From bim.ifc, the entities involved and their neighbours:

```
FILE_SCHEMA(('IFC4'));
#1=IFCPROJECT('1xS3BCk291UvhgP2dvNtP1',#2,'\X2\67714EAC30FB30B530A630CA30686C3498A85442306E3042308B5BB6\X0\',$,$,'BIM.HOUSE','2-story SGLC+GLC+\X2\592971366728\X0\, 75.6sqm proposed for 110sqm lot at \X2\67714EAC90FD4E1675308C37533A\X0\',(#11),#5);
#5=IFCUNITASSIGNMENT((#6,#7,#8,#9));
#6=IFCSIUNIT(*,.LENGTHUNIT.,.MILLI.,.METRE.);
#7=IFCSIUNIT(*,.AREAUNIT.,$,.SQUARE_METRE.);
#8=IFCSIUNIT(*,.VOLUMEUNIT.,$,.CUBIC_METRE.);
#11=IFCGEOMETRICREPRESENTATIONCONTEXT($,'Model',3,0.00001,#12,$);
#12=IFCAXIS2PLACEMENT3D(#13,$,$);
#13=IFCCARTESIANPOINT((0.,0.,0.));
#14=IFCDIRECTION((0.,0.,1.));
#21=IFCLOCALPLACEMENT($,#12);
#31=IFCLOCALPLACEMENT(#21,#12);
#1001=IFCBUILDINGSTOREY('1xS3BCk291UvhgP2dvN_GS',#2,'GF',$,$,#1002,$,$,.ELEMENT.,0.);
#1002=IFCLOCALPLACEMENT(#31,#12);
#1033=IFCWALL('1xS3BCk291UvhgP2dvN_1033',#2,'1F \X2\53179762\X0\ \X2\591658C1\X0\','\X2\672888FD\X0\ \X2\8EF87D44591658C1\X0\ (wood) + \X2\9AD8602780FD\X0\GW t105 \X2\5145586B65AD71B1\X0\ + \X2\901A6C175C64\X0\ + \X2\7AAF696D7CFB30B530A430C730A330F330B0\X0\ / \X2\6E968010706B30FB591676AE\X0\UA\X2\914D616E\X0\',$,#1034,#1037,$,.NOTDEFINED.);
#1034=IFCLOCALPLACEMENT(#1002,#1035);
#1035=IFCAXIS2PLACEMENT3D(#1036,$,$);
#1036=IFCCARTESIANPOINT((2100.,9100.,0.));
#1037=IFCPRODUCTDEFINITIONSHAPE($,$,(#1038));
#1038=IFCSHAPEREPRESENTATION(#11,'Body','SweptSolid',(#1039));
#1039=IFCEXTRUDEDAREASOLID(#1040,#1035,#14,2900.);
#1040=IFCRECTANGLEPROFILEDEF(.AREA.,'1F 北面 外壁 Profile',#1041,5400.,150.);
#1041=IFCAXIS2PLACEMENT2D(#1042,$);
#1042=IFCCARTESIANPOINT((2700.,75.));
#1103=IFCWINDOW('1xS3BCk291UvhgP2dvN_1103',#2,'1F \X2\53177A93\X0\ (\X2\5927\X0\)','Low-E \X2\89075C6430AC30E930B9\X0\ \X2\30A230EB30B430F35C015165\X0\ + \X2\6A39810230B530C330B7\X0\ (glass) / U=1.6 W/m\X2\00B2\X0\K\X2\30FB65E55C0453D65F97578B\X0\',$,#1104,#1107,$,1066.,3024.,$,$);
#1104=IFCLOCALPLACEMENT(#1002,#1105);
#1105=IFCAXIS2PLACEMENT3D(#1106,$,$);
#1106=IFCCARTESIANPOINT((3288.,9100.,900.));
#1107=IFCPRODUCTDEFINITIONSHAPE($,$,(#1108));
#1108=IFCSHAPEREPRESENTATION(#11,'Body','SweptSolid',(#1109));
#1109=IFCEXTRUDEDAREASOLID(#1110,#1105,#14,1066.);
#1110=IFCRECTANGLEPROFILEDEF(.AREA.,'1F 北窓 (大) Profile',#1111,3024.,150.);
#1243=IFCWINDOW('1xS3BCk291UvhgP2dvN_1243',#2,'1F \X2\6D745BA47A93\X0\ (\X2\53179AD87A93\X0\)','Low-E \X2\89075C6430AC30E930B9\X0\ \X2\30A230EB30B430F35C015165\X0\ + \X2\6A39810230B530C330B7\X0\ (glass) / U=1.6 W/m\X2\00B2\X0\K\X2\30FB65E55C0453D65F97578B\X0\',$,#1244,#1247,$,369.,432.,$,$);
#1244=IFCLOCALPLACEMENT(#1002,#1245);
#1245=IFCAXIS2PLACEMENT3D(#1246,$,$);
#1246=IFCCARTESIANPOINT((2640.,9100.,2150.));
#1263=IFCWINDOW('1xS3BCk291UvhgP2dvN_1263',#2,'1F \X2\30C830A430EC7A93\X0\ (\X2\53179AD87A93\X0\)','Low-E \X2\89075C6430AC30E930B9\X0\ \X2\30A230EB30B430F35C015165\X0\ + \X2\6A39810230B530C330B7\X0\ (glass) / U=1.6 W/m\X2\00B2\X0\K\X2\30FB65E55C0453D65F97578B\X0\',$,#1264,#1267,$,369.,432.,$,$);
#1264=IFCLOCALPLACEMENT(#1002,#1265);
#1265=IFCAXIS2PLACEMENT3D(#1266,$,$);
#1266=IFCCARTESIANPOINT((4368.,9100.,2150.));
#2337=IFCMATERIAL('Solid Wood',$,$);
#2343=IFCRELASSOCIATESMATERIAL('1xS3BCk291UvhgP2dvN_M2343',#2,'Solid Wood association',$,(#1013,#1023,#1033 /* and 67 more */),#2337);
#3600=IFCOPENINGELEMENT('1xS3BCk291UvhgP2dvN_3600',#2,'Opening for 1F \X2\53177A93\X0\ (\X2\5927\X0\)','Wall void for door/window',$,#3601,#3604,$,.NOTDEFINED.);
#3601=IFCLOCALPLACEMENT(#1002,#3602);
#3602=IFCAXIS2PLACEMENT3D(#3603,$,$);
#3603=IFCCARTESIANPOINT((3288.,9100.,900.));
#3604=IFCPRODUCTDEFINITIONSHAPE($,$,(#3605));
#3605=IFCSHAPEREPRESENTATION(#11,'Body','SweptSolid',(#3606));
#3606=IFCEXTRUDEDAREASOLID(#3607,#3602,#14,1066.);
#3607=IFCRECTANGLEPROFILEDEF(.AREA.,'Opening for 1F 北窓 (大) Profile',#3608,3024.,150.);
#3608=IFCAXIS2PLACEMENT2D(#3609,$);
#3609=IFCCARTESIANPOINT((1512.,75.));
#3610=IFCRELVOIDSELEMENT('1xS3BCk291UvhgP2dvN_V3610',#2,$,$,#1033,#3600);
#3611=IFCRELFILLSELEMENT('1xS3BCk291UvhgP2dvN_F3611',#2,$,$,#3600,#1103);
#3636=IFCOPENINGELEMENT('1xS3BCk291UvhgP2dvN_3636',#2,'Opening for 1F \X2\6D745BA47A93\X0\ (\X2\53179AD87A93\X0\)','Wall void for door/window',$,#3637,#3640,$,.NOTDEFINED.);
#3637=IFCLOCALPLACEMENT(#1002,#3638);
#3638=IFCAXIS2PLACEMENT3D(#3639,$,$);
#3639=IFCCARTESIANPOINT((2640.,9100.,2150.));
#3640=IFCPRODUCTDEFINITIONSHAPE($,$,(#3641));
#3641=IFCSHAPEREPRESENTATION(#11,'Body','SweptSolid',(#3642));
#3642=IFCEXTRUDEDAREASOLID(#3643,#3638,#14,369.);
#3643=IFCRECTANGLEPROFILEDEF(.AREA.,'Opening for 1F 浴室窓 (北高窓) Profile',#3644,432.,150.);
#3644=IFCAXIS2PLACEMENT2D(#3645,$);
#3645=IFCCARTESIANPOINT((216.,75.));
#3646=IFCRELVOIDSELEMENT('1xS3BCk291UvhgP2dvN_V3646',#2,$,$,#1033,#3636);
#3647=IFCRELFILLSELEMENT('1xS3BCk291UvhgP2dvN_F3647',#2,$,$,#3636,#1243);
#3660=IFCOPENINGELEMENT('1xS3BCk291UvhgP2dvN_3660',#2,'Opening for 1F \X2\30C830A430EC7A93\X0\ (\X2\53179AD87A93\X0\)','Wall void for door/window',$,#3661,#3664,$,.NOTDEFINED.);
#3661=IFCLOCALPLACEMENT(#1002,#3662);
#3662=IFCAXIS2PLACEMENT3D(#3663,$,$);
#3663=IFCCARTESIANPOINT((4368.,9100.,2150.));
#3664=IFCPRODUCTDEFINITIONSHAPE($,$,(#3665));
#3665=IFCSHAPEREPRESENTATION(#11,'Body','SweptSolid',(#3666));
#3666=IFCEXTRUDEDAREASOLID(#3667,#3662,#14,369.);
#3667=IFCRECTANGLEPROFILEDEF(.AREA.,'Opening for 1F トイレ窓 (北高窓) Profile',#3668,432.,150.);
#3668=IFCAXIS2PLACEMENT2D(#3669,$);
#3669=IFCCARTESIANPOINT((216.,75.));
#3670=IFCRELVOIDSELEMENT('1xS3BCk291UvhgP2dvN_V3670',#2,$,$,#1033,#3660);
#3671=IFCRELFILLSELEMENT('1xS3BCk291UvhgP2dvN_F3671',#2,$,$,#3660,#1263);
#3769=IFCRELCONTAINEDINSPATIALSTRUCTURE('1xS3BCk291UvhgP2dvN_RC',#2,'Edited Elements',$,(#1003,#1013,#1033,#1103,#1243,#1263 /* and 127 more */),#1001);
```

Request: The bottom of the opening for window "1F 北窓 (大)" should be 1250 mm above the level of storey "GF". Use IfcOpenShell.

```python
import numpy as np
import ifcopenshell
import ifcopenshell.api.geometry
import ifcopenshell.geom
import ifcopenshell.util.element
import ifcopenshell.util.placement
import ifcopenshell.util.shape
import ifcopenshell.util.unit

model = ifcopenshell.open("bim.ifc")
unit_scale = ifcopenshell.util.unit.calculate_unit_scale(model)

window = model.by_guid("1xS3BCk291UvhgP2dvN_1103")
opening = window.FillsVoids[0].RelatingOpeningElement
storey = ifcopenshell.util.element.get_container(window, ifc_class="IfcBuildingStorey")
level = ifcopenshell.util.placement.get_local_placement(storey.ObjectPlacement)[2, 3]

# The opening's origin need not be at the sill, so measure its lowest point.
shape = ifcopenshell.geom.create_shape(ifcopenshell.geom.settings(), opening)
bottom = ifcopenshell.util.shape.get_shape_bottom_elevation(shape, shape.geometry) / unit_scale
dz = level + 1.25 / unit_scale - bottom

shift = np.array([0.0, 0.0, dz])
# The window is not placed relative to its opening, so move both.
for product in (opening, window):
    matrix = ifcopenshell.util.placement.get_local_placement(product.ObjectPlacement)
    matrix[:3, 3] += shift
    ifcopenshell.api.geometry.edit_object_placement(model, product=product, matrix=matrix, is_si=False)

print(f"moved by {dz * unit_scale:+.3f} m")

model.write("bim-out.ifc")
```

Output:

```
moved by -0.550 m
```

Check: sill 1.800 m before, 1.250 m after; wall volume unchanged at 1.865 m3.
